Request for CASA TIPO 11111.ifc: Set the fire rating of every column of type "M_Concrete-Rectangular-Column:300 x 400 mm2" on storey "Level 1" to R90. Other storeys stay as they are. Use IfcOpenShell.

First a look at what the model holds.

```python
import ifcopenshell
import ifcopenshell.util.element

model = ifcopenshell.open("CASA TIPO 11111.ifc")
print(model.schema)
storey = next(s for s in model.by_type("IfcBuildingStorey") if s.Name == "Level 1")
columns = [e for e in ifcopenshell.util.element.get_decomposition(storey) if e.is_a("IfcColumn")]
seen = {}
for e in columns:
    element_type = ifcopenshell.util.element.get_type(e)
    key = (element_type.Name if element_type != e and element_type else None, ifcopenshell.util.element.get_pset(e, "Pset_ColumnCommon", "FireRating"))
    seen[key] = seen.get(key, 0) + 1
for (name, value), count in sorted(seen.items(), key=str):
    print(count, "x", name, "|", value)
```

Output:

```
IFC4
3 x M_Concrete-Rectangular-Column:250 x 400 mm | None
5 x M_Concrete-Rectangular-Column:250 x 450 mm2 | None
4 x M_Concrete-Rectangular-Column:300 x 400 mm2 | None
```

```python
import ifcopenshell
import ifcopenshell.api.pset
import ifcopenshell.util.element

model = ifcopenshell.open("CASA TIPO 11111.ifc")

storey = next(s for s in model.by_type("IfcBuildingStorey") if s.Name == "Level 1")
columns = [e for e in ifcopenshell.util.element.get_decomposition(storey) if e.is_a("IfcColumn")]

count = 0
for e in columns:
    element_type = ifcopenshell.util.element.get_type(e)
    if element_type in (None, e) or element_type.Name != "M_Concrete-Rectangular-Column:300 x 400 mm2":
        continue
    # add_pset returns the element's existing set when there is one.
    pset = ifcopenshell.api.pset.add_pset(model, product=e, name="Pset_ColumnCommon")
    ifcopenshell.api.pset.edit_pset(model, pset=pset, properties={"FireRating": "R90"})
    count += 1

print(count, "columns updated")

model.write("CASA TIPO 11111-out.ifc")
```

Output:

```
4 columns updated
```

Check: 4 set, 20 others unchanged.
